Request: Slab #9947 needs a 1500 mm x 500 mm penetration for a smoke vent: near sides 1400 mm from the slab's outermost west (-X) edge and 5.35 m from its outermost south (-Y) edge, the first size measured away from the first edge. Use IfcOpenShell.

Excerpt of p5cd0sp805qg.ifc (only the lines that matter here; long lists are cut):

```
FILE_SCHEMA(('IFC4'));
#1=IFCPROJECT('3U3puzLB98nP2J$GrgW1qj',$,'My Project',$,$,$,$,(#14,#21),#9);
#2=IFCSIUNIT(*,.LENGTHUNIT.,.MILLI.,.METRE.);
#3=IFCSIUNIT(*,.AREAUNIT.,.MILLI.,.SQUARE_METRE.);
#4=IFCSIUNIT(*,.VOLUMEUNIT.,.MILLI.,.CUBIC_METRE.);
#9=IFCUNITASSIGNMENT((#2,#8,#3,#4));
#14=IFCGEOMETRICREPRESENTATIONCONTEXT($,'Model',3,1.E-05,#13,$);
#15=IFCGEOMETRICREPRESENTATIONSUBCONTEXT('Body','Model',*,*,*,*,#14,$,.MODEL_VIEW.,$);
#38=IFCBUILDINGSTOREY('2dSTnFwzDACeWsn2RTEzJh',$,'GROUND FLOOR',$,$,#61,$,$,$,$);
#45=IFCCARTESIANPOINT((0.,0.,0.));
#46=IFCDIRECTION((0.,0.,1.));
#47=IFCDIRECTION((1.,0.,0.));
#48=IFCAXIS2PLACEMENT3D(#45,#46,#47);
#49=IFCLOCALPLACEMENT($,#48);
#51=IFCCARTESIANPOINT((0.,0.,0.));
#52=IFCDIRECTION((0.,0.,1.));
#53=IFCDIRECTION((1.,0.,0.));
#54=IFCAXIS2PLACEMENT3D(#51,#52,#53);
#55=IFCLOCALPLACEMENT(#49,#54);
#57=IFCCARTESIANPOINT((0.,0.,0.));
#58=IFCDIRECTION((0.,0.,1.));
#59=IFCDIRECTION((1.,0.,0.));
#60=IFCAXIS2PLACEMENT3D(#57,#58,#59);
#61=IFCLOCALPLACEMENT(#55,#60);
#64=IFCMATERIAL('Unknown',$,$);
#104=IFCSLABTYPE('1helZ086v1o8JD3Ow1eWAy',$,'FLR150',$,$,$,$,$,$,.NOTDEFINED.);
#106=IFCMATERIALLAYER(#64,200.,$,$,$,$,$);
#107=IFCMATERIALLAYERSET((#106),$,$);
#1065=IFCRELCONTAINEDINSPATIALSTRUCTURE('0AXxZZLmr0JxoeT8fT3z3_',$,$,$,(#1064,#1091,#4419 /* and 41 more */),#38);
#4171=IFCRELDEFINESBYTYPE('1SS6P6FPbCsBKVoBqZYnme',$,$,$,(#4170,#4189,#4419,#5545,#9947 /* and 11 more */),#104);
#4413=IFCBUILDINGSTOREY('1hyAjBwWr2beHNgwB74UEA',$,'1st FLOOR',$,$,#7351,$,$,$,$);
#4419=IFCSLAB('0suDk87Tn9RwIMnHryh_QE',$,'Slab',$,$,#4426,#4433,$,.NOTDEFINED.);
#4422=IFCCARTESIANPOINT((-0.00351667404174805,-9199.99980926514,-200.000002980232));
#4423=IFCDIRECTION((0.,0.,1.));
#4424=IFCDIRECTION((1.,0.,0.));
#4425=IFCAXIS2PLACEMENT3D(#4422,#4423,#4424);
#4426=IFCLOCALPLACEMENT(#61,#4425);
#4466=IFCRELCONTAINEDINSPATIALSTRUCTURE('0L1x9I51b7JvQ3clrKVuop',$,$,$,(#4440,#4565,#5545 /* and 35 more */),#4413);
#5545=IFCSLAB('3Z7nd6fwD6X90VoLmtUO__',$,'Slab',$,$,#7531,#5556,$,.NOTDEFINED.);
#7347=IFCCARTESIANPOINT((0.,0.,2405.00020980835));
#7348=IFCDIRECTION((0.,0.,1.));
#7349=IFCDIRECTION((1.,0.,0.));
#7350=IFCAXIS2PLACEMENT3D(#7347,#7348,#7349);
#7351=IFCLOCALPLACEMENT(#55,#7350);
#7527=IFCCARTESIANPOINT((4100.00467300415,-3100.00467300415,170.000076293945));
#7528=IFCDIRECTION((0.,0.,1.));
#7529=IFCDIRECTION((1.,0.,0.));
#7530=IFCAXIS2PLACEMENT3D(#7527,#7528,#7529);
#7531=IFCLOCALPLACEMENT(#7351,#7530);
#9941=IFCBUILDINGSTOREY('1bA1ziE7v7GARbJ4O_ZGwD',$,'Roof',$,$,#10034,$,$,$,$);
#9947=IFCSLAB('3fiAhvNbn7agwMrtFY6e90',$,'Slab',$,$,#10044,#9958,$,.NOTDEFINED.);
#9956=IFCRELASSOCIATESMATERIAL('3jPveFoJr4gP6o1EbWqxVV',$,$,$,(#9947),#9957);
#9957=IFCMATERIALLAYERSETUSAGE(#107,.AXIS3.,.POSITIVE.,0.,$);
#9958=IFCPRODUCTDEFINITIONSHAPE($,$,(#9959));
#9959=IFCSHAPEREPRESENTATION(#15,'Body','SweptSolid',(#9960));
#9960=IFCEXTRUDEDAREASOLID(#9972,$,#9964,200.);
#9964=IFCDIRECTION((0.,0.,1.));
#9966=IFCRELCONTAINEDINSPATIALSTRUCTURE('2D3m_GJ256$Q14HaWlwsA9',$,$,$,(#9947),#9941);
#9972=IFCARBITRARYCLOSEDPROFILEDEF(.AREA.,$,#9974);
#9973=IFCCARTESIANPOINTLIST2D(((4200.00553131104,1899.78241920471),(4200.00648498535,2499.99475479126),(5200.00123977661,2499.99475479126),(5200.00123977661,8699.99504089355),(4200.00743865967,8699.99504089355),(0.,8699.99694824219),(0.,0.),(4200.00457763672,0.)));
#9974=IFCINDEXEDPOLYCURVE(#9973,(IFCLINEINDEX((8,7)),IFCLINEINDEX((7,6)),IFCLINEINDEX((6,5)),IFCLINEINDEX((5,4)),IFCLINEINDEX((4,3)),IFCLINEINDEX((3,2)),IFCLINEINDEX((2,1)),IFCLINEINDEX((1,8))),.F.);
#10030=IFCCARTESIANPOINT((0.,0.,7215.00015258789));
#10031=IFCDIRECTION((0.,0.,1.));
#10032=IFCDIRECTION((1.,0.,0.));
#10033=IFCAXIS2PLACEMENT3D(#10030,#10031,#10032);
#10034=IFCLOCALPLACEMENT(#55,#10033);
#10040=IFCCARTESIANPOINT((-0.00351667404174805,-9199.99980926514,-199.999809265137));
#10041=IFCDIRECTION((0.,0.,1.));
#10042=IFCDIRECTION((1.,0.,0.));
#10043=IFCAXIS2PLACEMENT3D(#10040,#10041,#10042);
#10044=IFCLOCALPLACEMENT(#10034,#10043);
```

```python
import numpy as np
import ifcopenshell
import ifcopenshell.api.feature
import ifcopenshell.api.geometry
import ifcopenshell.api.root
import ifcopenshell.geom
import ifcopenshell.util.placement
import ifcopenshell.util.representation
import ifcopenshell.util.shape
import ifcopenshell.util.unit

model = ifcopenshell.open("p5cd0sp805qg.ifc")
unit_scale = ifcopenshell.util.unit.calculate_unit_scale(model)
settings = ifcopenshell.geom.settings()


def volume(element):
    """Net volume in cubic metres, openings subtracted."""
    shape = ifcopenshell.geom.create_shape(settings, element)
    return ifcopenshell.util.shape.get_volume(shape.geometry)


slab = model.by_id(9947)
before = volume(slab)

# Extent in the slab's own axes, in metres. The edges named are its -X and -Y sides.
slab_shape = ifcopenshell.geom.create_shape(settings, slab)
vertices = ifcopenshell.util.shape.get_vertices(slab_shape.geometry)
x_min, y_min, bottom = vertices.min(axis=0)
top = vertices[:, 2].max()

opening = ifcopenshell.api.root.create_entity(model, ifc_class="IfcOpeningElement", name="Smoke vent opening", predefined_type="OPENING")
context = ifcopenshell.util.representation.get_context(model, "Model", "Body", "MODEL_VIEW")
width, depth = 1.5, 0.5
outline = [(0.0, 0.0), (width, 0.0), (width, depth), (0.0, depth), (0.0, 0.0)]
# Overshoot both faces by 50 mm so the cut is clean.
shape = ifcopenshell.api.geometry.add_slab_representation(
    model, context=context, depth=top - bottom + 0.1, polyline=outline
)
ifcopenshell.api.geometry.assign_representation(model, product=opening, representation=shape)

matrix = ifcopenshell.util.placement.get_local_placement(slab.ObjectPlacement)
matrix[:, 3] = matrix @ np.append(np.array([x_min + 1.4, y_min + 5.35, bottom - 0.05]) / unit_scale, 1.0)
ifcopenshell.api.geometry.edit_object_placement(model, product=opening, matrix=matrix, is_si=False)
ifcopenshell.api.feature.add_feature(model, feature=opening, element=slab)

after = volume(slab)

print(f"slab volume {before:.3f} -> {after:.3f} m3")

model.write("p5cd0sp805qg-out.ifc")
```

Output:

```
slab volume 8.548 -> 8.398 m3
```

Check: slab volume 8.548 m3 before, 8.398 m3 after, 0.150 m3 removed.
